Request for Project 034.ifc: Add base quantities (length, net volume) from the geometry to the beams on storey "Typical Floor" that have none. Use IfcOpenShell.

First a look at what the model holds.

```python
import ifcopenshell
import ifcopenshell.util.element
import ifcopenshell.util.unit

model = ifcopenshell.open("Project 034.ifc")
print(model.schema)
for unit_type in ("LENGTHUNIT", "AREAUNIT", "VOLUMEUNIT"):
    print(unit_type, ifcopenshell.util.unit.calculate_unit_scale(model, unit_type))
storey = next(s for s in model.by_type("IfcBuildingStorey") if s.Name == "Typical Floor")
beams = [e for e in ifcopenshell.util.element.get_decomposition(storey) if e.is_a("IfcBeam")]
for e in sorted(beams, key=lambda e: e.id()):
    print(e.id(), e.is_a(), e.Name, list(ifcopenshell.util.element.get_psets(e, qtos_only=True)), sep=" | ")
```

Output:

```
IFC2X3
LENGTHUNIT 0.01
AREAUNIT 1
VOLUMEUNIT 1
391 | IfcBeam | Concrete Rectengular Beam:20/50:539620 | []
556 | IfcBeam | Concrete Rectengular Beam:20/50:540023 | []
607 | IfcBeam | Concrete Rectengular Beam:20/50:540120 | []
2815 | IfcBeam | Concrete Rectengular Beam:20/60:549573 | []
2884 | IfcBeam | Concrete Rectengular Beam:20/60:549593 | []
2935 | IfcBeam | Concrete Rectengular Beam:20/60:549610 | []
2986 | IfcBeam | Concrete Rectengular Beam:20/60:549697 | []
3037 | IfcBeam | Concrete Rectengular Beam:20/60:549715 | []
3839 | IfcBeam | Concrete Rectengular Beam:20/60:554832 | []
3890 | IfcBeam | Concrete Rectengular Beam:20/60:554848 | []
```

```python
import ifcopenshell
import ifcopenshell.api.pset
import ifcopenshell.geom
import ifcopenshell.util.element
import ifcopenshell.util.shape
import ifcopenshell.util.unit

model = ifcopenshell.open("Project 034.ifc")
unit_scale = ifcopenshell.util.unit.calculate_unit_scale(model)
volume_scale = ifcopenshell.util.unit.calculate_unit_scale(model, "VOLUMEUNIT")
settings = ifcopenshell.geom.settings()

storey = next(s for s in model.by_type("IfcBuildingStorey") if s.Name == "Typical Floor")
beams = [e for e in ifcopenshell.util.element.get_decomposition(storey) if e.is_a("IfcBeam")]

for e in sorted(beams, key=lambda e: e.id()):
    if ifcopenshell.util.element.get_psets(e, qtos_only=True, should_inherit=False):
        continue
    # Geometry comes back in metres, in the element's own axes.
    shape = ifcopenshell.geom.create_shape(settings, e)
    values = {
        "Length": ifcopenshell.util.shape.get_max_xyz(shape.geometry) / unit_scale,
        "NetVolume": ifcopenshell.util.shape.get_volume(shape.geometry) / volume_scale,
    }
    qto = ifcopenshell.api.pset.add_qto(model, product=e, name="BaseQuantities")
    ifcopenshell.api.pset.edit_qto(model, qto=qto, properties=values)
    print(e.id(), {k: round(v, 3) for k, v in values.items()})

model.write("Project 034_updated.ifc")
```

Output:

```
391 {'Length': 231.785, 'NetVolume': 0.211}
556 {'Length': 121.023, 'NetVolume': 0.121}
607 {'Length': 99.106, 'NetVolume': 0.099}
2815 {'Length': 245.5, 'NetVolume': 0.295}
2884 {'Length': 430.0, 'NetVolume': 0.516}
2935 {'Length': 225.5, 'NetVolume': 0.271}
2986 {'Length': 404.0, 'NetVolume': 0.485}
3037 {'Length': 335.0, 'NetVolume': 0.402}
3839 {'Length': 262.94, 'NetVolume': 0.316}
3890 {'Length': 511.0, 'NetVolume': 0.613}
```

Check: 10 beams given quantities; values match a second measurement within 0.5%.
